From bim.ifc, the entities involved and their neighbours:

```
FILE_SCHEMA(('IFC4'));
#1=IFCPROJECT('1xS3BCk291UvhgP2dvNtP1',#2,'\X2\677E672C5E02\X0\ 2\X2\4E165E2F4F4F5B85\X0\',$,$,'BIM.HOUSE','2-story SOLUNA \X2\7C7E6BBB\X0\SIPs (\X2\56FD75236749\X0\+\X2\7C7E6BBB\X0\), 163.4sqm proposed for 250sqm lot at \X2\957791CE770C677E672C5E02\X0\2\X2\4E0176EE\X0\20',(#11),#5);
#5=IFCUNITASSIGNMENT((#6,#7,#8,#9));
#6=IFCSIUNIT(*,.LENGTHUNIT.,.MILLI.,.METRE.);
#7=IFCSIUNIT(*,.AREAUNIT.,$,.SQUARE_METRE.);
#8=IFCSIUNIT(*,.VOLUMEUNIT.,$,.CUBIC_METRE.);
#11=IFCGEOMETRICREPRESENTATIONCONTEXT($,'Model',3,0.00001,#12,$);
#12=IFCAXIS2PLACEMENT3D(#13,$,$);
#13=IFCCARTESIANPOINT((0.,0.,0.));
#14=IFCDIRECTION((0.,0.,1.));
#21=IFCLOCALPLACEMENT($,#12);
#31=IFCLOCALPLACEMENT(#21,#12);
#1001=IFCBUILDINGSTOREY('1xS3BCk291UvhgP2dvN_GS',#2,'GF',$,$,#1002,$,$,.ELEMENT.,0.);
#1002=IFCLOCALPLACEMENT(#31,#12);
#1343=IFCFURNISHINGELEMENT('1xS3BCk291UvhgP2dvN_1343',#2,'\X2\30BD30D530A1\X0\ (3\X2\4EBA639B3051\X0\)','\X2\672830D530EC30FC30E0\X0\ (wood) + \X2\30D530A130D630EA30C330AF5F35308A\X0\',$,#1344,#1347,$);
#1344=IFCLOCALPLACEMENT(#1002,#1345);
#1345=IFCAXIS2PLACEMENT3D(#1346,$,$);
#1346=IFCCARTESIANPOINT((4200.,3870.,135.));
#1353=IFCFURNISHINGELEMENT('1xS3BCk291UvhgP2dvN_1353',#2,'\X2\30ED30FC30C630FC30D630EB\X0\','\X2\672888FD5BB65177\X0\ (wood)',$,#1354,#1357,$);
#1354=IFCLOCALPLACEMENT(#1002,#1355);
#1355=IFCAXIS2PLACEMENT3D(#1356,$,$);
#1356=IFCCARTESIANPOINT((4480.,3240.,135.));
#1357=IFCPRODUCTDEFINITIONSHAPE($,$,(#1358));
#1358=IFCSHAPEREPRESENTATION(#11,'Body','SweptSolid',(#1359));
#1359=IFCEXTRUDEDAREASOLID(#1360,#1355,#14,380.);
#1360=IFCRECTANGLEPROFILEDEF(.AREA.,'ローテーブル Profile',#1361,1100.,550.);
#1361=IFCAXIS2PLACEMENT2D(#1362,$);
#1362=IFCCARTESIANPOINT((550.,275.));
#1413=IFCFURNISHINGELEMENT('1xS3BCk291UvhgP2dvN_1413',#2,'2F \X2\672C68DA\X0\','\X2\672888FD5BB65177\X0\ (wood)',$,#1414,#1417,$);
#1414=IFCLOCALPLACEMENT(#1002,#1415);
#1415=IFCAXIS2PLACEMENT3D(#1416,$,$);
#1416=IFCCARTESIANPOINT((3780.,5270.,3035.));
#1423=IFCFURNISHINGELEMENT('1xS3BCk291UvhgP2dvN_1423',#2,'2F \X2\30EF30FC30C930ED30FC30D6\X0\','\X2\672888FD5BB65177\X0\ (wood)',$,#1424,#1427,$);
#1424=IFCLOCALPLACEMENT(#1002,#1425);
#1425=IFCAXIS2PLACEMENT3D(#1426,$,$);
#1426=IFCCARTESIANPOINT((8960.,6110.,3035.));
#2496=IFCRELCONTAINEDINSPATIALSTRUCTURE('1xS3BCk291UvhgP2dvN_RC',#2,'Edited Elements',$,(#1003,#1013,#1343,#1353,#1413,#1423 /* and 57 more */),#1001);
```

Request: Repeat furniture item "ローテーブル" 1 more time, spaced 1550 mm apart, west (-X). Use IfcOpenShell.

```python
import numpy as np
import ifcopenshell
import ifcopenshell.api.geometry
import ifcopenshell.api.root
import ifcopenshell.util.element
import ifcopenshell.util.placement

model = ifcopenshell.open("bim.ifc")


def reuse_history(source, copy):
    """copy_class also copies each property set's owner history, people and application; keep the originals."""
    for rel in copy.IsDefinedBy:
        if rel.is_a("IfcRelDefinesByProperties") and (history := rel.RelatingPropertyDefinition.OwnerHistory):
            rel.RelatingPropertyDefinition.OwnerHistory = source.OwnerHistory
            ifcopenshell.util.element.remove_deep2(model, history)


source = model.by_guid("1xS3BCk291UvhgP2dvN_1353")
base = ifcopenshell.util.placement.get_local_placement(source.ObjectPlacement)
step = np.array([-1.0, 0.0, 0.0]) * 1550.0

for i in range(1, 2):
    copy = ifcopenshell.api.root.copy_class(model, product=source)
    copy.Representation = ifcopenshell.util.element.copy_deep(
        model, source.Representation, exclude=["IfcGeometricRepresentationContext", "IfcRepresentationMap"]
    )
    reuse_history(source, copy)
    matrix = base.copy()
    matrix[:3, 3] += i * step
    print("added at", matrix[:3, 3].round(3) + 0.0)
    ifcopenshell.api.geometry.edit_object_placement(model, product=copy, matrix=matrix, is_si=False)

model.write("bim_rev.ifc")
```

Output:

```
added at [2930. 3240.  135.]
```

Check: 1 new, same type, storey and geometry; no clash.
